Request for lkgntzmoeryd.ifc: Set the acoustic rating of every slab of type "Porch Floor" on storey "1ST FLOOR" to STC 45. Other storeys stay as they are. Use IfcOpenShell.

First a look at what the model holds.

```python
import ifcopenshell
import ifcopenshell.util.element

model = ifcopenshell.open("lkgntzmoeryd.ifc")
print(model.schema)
storey = next(s for s in model.by_type("IfcBuildingStorey") if s.Name == "1ST FLOOR")
slabs = [e for e in ifcopenshell.util.element.get_decomposition(storey) if e.is_a("IfcSlab")]
seen = {}
for e in slabs:
    element_type = ifcopenshell.util.element.get_type(e)
    key = (element_type.Name if element_type != e and element_type else None, ifcopenshell.util.element.get_pset(e, "Pset_SlabCommon", "AcousticRating"))
    seen[key] = seen.get(key, 0) + 1
for (name, value), count in sorted(seen.items(), key=str):
    print(count, "x", name, "|", value)
```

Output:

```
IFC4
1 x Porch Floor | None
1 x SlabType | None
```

```python
import ifcopenshell
import ifcopenshell.api.pset
import ifcopenshell.util.element

model = ifcopenshell.open("lkgntzmoeryd.ifc")

storey = next(s for s in model.by_type("IfcBuildingStorey") if s.Name == "1ST FLOOR")
slabs = [e for e in ifcopenshell.util.element.get_decomposition(storey) if e.is_a("IfcSlab")]

count = 0
for e in slabs:
    element_type = ifcopenshell.util.element.get_type(e)
    if element_type in (None, e) or element_type.Name != "Porch Floor":
        continue
    # add_pset returns the element's existing set when there is one.
    pset = ifcopenshell.api.pset.add_pset(model, product=e, name="Pset_SlabCommon")
    ifcopenshell.api.pset.edit_pset(model, pset=pset, properties={"AcousticRating": "STC 45"})
    count += 1

print(count, "slabs updated")

model.write("lkgntzmoeryd_edited.ifc")
```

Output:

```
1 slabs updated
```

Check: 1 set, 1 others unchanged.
